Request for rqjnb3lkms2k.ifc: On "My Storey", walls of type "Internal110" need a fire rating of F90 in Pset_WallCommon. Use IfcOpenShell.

First a look at what the model holds.

```python
import ifcopenshell
import ifcopenshell.util.element

model = ifcopenshell.open("rqjnb3lkms2k.ifc")
print(model.schema)
storey = next(s for s in model.by_type("IfcBuildingStorey") if s.Name == "My Storey")
walls = [e for e in ifcopenshell.util.element.get_decomposition(storey) if e.is_a("IfcWall")]
seen = {}
for e in walls:
    element_type = ifcopenshell.util.element.get_type(e)
    key = (element_type.Name if element_type != e and element_type else None, ifcopenshell.util.element.get_pset(e, "Pset_WallCommon", "FireRating"))
    seen[key] = seen.get(key, 0) + 1
for (name, value), count in sorted(seen.items(), key=str):
    print(count, "x", name, "|", value)
```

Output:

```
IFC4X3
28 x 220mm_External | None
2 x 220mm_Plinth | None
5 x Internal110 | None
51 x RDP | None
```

```python
import ifcopenshell
import ifcopenshell.api.pset
import ifcopenshell.util.element

model = ifcopenshell.open("rqjnb3lkms2k.ifc")

storey = next(s for s in model.by_type("IfcBuildingStorey") if s.Name == "My Storey")
walls = [e for e in ifcopenshell.util.element.get_decomposition(storey) if e.is_a("IfcWall")]

count = 0
for e in walls:
    element_type = ifcopenshell.util.element.get_type(e)
    if element_type in (None, e) or element_type.Name != "Internal110":
        continue
    # add_pset returns the element's existing set when there is one.
    pset = ifcopenshell.api.pset.add_pset(model, product=e, name="Pset_WallCommon")
    ifcopenshell.api.pset.edit_pset(model, pset=pset, properties={"FireRating": "F90"})
    count += 1

print(count, "walls updated")

model.write("rqjnb3lkms2k_updated.ifc")
```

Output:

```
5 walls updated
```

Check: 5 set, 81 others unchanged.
